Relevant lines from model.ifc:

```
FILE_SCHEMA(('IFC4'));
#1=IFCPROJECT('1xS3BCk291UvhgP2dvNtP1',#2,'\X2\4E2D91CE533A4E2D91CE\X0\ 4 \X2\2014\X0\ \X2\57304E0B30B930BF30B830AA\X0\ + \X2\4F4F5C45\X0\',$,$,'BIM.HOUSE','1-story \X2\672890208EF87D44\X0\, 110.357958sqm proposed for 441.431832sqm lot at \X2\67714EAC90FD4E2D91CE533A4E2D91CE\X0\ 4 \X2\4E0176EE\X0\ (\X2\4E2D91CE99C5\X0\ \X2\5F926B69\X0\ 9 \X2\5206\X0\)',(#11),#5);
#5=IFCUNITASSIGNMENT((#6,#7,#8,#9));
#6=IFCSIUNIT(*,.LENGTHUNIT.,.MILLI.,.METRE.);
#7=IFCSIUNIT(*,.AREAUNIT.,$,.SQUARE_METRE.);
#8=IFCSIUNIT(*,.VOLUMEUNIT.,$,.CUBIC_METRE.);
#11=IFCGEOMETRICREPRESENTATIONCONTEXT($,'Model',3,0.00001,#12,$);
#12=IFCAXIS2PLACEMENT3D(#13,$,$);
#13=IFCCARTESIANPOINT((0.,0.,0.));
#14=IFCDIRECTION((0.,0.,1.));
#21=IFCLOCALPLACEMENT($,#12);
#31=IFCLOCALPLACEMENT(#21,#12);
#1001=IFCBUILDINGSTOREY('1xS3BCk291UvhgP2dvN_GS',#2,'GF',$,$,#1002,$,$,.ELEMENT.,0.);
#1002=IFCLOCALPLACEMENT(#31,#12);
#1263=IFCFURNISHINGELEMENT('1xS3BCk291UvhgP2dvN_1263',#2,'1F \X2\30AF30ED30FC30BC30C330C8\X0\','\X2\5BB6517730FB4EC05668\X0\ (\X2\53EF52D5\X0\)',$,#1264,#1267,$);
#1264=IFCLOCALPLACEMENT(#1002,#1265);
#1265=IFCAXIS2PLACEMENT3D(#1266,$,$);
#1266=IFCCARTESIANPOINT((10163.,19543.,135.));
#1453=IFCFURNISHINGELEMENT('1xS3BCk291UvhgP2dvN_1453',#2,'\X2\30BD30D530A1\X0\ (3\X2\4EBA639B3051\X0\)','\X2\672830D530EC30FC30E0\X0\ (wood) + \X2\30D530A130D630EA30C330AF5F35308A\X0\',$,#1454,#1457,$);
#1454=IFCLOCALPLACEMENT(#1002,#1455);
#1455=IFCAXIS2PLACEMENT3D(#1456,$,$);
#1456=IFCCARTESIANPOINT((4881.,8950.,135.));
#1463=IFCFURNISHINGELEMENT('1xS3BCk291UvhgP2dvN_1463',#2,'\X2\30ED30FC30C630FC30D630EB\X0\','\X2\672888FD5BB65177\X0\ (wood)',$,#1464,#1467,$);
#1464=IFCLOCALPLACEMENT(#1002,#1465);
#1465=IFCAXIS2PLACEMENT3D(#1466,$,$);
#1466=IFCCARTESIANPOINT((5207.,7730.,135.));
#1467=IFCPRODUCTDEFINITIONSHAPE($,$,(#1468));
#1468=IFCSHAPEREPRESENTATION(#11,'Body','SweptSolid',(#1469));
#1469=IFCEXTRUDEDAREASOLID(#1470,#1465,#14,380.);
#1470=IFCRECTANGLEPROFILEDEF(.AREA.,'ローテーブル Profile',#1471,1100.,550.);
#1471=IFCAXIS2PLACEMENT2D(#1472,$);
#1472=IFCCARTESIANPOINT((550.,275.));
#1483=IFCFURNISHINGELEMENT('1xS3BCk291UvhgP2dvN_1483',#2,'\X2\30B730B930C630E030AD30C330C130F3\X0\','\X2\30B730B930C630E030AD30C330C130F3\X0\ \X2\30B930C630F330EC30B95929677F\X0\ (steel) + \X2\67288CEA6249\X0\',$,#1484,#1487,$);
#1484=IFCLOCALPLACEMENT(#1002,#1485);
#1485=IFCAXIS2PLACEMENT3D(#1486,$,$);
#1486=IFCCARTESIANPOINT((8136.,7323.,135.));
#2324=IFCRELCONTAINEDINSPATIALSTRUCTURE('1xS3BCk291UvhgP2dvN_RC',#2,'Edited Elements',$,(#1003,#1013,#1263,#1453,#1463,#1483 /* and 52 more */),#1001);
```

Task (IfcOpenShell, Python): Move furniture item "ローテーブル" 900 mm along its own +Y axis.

```python
import ifcopenshell
import ifcopenshell.api.geometry
import ifcopenshell.util.placement

model = ifcopenshell.open("model.ifc")

item = model.by_guid("1xS3BCk291UvhgP2dvN_1463")
matrix = ifcopenshell.util.placement.get_local_placement(item.ObjectPlacement)
matrix[:3, 3] += matrix[:3, 1] * 900.0
ifcopenshell.api.geometry.edit_object_placement(model, product=item, matrix=matrix, is_si=False)

print(ifcopenshell.util.placement.get_local_placement(item.ObjectPlacement).round(3) + 0.0)

model.write("model-out.ifc")
```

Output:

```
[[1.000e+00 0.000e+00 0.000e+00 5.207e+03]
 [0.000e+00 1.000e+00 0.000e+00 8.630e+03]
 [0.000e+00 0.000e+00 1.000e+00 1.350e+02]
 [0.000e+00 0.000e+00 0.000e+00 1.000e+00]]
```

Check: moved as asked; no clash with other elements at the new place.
